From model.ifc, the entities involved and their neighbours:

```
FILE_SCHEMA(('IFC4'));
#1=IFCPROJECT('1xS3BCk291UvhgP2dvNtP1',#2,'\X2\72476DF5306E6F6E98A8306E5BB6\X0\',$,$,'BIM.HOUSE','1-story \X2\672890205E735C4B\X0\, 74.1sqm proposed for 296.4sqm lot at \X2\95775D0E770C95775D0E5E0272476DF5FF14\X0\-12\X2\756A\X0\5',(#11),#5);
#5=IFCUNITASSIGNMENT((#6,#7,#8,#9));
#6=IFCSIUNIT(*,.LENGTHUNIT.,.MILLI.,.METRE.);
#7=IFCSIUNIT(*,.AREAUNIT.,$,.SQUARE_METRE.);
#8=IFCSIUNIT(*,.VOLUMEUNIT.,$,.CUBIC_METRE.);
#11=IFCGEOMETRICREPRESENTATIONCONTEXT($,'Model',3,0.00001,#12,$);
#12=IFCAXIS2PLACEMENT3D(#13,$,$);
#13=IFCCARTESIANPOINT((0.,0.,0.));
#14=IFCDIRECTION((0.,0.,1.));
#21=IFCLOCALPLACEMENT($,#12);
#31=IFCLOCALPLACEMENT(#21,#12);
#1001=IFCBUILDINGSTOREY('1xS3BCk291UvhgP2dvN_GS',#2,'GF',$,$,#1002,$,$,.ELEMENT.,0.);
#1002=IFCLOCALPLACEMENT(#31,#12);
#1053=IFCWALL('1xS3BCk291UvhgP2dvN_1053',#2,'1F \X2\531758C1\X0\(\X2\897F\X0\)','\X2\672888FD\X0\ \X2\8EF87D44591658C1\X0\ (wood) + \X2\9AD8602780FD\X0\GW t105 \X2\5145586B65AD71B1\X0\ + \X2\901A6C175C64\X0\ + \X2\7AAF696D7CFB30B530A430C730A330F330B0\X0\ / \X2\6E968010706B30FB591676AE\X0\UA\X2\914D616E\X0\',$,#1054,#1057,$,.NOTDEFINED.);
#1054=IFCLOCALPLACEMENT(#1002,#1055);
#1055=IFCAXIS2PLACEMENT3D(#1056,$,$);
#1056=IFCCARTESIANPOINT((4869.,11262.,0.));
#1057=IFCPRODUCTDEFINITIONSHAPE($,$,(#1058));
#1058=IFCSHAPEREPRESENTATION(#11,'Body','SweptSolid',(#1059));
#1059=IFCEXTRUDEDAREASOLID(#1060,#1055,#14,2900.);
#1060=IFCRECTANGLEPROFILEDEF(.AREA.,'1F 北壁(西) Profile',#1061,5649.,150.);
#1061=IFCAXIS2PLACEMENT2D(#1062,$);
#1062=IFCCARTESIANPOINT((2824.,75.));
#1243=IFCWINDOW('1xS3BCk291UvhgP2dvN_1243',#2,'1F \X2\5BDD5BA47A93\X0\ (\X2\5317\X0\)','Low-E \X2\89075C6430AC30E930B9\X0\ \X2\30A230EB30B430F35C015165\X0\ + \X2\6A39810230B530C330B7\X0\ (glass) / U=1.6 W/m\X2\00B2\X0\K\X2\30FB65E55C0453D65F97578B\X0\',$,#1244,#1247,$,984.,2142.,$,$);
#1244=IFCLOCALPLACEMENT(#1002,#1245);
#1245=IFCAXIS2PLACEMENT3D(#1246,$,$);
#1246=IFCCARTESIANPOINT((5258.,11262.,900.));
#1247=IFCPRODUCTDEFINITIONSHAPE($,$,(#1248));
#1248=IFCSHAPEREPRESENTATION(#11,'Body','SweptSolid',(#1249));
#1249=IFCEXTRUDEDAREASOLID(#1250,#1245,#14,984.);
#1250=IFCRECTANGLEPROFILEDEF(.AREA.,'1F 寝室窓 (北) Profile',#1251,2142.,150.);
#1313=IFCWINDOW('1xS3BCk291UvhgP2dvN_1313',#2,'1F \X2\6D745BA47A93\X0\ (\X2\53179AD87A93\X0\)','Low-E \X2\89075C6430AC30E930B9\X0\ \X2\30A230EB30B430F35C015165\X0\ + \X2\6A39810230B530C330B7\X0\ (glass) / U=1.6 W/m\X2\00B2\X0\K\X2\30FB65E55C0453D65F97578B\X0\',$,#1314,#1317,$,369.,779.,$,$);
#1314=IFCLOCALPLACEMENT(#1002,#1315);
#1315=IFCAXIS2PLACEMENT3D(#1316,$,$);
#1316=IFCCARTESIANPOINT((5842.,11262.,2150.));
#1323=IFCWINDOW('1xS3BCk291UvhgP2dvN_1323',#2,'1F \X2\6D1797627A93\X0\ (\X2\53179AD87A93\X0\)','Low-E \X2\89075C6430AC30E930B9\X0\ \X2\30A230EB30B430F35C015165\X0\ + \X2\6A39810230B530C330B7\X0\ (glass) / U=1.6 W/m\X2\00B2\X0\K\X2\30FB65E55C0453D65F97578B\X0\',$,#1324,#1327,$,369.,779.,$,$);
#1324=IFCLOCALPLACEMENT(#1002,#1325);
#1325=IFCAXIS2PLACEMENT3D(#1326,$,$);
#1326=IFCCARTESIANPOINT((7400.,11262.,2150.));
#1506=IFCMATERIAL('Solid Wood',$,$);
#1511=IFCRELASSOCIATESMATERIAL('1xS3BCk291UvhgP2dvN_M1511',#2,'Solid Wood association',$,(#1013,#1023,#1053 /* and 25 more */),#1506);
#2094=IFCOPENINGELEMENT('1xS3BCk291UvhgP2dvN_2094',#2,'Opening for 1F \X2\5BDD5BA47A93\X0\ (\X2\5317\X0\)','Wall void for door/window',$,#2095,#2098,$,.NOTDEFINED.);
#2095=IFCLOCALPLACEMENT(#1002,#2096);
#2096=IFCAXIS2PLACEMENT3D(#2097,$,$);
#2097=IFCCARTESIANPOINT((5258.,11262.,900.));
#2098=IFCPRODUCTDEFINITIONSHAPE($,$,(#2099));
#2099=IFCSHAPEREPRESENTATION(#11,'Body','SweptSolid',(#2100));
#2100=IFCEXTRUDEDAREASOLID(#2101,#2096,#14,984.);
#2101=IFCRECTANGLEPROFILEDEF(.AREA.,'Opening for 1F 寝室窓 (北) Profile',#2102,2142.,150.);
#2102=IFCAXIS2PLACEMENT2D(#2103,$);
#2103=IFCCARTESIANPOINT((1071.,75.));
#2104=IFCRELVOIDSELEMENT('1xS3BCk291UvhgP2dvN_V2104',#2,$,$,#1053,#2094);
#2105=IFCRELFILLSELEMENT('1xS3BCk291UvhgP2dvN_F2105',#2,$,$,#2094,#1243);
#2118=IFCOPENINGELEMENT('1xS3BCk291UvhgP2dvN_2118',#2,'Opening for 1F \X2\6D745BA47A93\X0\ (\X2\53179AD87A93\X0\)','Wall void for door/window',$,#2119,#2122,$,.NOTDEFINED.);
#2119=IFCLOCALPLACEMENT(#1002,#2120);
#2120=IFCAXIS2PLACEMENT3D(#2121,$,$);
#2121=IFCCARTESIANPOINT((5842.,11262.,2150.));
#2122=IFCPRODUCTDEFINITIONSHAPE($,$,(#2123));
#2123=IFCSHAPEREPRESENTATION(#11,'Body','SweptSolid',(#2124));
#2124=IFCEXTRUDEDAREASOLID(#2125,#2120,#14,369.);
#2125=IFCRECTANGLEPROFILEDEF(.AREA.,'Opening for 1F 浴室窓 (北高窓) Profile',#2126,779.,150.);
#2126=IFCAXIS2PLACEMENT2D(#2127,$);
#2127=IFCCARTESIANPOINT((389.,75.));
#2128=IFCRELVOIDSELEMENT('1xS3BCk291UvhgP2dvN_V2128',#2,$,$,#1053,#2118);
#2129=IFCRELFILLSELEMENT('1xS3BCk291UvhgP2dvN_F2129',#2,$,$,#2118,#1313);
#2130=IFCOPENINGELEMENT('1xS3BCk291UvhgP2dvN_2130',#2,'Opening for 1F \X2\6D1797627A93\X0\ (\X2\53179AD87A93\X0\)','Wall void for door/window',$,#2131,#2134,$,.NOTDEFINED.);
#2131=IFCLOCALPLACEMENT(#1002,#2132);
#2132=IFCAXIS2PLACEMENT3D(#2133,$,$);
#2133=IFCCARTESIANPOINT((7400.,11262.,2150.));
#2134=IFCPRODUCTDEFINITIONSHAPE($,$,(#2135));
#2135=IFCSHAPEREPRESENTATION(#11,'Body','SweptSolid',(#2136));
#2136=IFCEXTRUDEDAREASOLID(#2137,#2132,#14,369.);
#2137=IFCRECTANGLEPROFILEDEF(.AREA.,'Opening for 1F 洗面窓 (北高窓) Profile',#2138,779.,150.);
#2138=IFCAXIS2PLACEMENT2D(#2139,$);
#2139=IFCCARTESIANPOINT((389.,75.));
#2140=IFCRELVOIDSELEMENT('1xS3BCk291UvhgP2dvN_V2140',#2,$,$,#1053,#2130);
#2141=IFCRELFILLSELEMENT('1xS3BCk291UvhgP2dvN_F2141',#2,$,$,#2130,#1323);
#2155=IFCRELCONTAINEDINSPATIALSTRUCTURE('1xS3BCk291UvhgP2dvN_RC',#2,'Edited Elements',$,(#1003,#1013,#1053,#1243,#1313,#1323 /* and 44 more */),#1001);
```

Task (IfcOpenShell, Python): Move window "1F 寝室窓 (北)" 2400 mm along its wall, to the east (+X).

```python
import ifcopenshell
import ifcopenshell.api.geometry
import ifcopenshell.util.placement
import ifcopenshell.util.unit

model = ifcopenshell.open("model.ifc")
unit_scale = ifcopenshell.util.unit.calculate_unit_scale(model)

window = model.by_id(1243)
opening = window.FillsVoids[0].RelatingOpeningElement
wall = opening.VoidsElements[0].RelatingBuildingElement

wall_matrix = ifcopenshell.util.placement.get_local_placement(wall.ObjectPlacement)
shift = wall_matrix[:3, 0] * 2.4 / unit_scale
before = ifcopenshell.util.placement.get_local_placement(window.ObjectPlacement)[:3, 3].copy()

# The window is not placed relative to its opening, so move both.
for product in (opening, window):
    matrix = ifcopenshell.util.placement.get_local_placement(product.ObjectPlacement)
    matrix[:3, 3] += shift
    ifcopenshell.api.geometry.edit_object_placement(model, product=product, matrix=matrix, is_si=False)

after = ifcopenshell.util.placement.get_local_placement(window.ObjectPlacement)[:3, 3]
print("window moved by", (after - before).round(3) + 0.0)

model.write("model_v2.ifc")
```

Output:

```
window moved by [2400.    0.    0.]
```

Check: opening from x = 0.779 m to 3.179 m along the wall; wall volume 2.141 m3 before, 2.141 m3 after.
